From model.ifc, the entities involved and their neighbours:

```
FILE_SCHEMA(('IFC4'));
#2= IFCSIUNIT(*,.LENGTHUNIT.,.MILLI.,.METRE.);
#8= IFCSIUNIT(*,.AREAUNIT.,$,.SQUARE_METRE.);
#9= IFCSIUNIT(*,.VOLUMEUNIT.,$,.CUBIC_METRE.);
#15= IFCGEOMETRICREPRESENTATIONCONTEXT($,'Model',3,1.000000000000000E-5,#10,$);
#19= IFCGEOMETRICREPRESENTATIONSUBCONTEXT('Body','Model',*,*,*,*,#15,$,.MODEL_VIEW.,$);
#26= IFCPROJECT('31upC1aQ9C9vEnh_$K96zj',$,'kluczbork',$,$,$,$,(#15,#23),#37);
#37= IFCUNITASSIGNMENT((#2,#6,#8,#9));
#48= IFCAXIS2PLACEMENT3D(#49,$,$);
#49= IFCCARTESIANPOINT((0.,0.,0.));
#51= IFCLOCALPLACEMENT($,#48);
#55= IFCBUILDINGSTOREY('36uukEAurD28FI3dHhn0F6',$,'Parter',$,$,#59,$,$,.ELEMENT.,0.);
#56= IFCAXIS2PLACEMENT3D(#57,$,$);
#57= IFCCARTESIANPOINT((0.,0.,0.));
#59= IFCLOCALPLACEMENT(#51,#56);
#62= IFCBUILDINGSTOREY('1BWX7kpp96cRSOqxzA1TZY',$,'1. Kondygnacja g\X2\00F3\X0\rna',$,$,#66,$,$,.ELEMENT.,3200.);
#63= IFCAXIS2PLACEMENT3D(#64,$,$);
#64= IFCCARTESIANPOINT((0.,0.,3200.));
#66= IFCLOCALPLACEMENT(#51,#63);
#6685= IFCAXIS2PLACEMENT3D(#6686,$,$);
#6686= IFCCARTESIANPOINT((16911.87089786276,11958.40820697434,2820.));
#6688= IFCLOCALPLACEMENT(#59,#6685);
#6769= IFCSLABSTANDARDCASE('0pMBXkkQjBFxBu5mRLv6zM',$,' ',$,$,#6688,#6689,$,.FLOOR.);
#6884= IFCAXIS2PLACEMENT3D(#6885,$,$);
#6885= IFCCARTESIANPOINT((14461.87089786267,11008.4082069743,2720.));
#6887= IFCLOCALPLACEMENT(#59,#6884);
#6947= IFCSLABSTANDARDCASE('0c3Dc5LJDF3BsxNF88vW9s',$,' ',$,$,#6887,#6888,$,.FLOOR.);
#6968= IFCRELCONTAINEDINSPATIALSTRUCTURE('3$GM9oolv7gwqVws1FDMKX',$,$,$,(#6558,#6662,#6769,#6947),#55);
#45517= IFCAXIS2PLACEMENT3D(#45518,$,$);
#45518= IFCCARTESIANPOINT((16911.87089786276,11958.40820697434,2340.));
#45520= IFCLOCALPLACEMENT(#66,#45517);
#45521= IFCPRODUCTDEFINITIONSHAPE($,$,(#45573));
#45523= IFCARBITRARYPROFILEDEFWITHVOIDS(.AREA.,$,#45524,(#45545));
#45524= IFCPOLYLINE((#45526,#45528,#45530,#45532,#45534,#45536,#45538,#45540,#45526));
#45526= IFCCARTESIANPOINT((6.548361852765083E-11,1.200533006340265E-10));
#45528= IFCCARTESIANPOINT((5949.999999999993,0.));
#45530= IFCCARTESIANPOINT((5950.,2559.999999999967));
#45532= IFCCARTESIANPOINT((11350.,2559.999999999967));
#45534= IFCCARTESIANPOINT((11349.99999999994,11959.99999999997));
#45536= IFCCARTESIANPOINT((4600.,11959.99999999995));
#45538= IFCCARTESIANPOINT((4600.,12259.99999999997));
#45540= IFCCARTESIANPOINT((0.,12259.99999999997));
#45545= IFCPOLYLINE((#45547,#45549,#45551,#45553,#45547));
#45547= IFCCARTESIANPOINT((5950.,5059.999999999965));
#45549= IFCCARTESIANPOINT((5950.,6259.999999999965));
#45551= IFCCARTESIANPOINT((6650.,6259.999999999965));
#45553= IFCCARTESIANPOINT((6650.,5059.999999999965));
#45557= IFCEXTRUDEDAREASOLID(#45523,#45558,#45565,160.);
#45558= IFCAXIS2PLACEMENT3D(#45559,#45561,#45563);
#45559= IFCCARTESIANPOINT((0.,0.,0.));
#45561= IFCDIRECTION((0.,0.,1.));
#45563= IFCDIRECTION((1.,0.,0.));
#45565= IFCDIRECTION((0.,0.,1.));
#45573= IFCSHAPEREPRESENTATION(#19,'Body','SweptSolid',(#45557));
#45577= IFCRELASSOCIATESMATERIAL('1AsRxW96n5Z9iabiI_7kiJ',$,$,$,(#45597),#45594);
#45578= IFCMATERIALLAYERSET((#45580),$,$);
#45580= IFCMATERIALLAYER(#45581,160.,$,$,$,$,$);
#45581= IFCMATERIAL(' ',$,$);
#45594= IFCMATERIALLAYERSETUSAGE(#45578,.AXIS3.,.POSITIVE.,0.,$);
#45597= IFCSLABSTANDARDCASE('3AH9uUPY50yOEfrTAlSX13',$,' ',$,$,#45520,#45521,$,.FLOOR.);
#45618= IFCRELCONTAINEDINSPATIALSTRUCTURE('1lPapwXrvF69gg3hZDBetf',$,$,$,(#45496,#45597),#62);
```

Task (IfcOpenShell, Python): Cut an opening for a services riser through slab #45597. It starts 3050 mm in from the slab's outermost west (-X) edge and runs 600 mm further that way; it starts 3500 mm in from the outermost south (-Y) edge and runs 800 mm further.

```python
import numpy as np
import ifcopenshell
import ifcopenshell.api.feature
import ifcopenshell.api.geometry
import ifcopenshell.api.root
import ifcopenshell.geom
import ifcopenshell.util.placement
import ifcopenshell.util.representation
import ifcopenshell.util.shape
import ifcopenshell.util.unit

model = ifcopenshell.open("model.ifc")
unit_scale = ifcopenshell.util.unit.calculate_unit_scale(model)
settings = ifcopenshell.geom.settings()


def volume(element):
    """Net volume in cubic metres, openings subtracted."""
    shape = ifcopenshell.geom.create_shape(settings, element)
    return ifcopenshell.util.shape.get_volume(shape.geometry)


slab = model.by_guid("3AH9uUPY50yOEfrTAlSX13")
before = volume(slab)

# Extent in the slab's own axes, in metres. The edges named are its -X and -Y sides.
slab_shape = ifcopenshell.geom.create_shape(settings, slab)
vertices = ifcopenshell.util.shape.get_vertices(slab_shape.geometry)
x_min, y_min, bottom = vertices.min(axis=0)
top = vertices[:, 2].max()

opening = ifcopenshell.api.root.create_entity(model, ifc_class="IfcOpeningElement", name="Services riser opening", predefined_type="OPENING")
context = ifcopenshell.util.representation.get_context(model, "Model", "Body", "MODEL_VIEW")
width, depth = 0.6, 0.8
outline = [(0.0, 0.0), (width, 0.0), (width, depth), (0.0, depth), (0.0, 0.0)]
# Overshoot both faces by 50 mm so the cut is clean.
shape = ifcopenshell.api.geometry.add_slab_representation(
    model, context=context, depth=top - bottom + 0.1, polyline=outline
)
ifcopenshell.api.geometry.assign_representation(model, product=opening, representation=shape)

matrix = ifcopenshell.util.placement.get_local_placement(slab.ObjectPlacement)
matrix[:, 3] = matrix @ np.append(np.array([x_min + 3.05, y_min + 3.5, bottom - 0.05]) / unit_scale, 1.0)
ifcopenshell.api.geometry.edit_object_placement(model, product=opening, matrix=matrix, is_si=False)
ifcopenshell.api.feature.add_feature(model, feature=opening, element=slab)

after = volume(slab)

print(f"slab volume {before:.3f} -> {after:.3f} m3")

model.write("model-out.ifc")
```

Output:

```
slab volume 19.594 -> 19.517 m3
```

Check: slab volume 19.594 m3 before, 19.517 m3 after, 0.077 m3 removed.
